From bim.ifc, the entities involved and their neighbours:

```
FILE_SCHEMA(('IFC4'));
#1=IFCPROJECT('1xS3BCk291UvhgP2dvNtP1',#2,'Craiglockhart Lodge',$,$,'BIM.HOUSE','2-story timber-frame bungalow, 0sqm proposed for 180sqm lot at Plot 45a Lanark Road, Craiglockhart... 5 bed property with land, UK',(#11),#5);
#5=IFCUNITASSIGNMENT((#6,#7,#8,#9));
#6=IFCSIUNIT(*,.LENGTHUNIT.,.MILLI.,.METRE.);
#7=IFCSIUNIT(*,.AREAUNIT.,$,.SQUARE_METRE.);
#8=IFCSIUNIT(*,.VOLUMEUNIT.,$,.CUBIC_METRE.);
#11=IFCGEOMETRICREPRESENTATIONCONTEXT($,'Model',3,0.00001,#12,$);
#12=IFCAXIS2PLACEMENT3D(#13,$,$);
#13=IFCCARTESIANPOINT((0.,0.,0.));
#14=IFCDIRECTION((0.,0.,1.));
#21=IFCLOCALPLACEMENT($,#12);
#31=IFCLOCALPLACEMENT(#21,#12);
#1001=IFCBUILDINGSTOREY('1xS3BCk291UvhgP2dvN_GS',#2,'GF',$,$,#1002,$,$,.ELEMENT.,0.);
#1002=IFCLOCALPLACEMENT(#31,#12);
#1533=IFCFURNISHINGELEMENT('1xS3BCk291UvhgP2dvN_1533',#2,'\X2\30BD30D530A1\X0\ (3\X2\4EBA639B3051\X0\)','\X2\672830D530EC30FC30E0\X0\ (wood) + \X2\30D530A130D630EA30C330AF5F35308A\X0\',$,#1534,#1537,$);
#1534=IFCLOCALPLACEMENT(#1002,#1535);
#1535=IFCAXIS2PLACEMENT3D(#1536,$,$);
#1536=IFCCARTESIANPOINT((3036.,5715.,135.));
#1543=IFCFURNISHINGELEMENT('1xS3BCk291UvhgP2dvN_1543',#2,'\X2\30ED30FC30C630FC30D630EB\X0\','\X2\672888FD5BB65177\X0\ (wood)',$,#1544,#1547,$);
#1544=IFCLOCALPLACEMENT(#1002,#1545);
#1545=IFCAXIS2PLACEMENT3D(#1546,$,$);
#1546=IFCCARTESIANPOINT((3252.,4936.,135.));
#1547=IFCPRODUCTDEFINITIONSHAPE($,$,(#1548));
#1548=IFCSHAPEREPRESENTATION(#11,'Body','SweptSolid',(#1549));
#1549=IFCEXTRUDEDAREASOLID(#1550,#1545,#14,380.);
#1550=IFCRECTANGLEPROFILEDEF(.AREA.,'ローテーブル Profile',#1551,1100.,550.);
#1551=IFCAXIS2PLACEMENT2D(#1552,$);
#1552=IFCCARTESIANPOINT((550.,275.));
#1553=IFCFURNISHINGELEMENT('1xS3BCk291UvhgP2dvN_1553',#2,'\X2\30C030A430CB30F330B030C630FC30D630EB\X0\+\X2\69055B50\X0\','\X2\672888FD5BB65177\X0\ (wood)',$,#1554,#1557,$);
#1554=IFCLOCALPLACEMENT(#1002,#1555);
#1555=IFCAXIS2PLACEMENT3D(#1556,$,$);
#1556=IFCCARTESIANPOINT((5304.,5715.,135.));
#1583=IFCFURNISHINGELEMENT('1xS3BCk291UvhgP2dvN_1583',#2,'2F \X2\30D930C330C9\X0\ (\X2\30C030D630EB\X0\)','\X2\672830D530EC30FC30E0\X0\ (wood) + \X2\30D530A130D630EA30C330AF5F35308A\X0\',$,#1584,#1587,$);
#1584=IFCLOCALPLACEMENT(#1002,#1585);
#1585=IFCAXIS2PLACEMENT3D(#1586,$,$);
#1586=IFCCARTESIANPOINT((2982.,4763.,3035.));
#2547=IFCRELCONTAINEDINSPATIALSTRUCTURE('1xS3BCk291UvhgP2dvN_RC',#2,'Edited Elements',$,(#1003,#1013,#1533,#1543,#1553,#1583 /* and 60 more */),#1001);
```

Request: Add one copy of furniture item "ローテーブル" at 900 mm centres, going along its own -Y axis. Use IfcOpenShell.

```python
import ifcopenshell
import ifcopenshell.api.geometry
import ifcopenshell.api.root
import ifcopenshell.util.element
import ifcopenshell.util.placement

model = ifcopenshell.open("bim.ifc")


def reuse_history(source, copy):
    """copy_class also copies each property set's owner history, people and application; keep the originals."""
    for rel in copy.IsDefinedBy:
        if rel.is_a("IfcRelDefinesByProperties") and (history := rel.RelatingPropertyDefinition.OwnerHistory):
            rel.RelatingPropertyDefinition.OwnerHistory = source.OwnerHistory
            ifcopenshell.util.element.remove_deep2(model, history)


source = model.by_id(1543)
base = ifcopenshell.util.placement.get_local_placement(source.ObjectPlacement)
step = -base[:3, 1] * 900.0

for i in range(1, 2):
    copy = ifcopenshell.api.root.copy_class(model, product=source)
    copy.Representation = ifcopenshell.util.element.copy_deep(
        model, source.Representation, exclude=["IfcGeometricRepresentationContext", "IfcRepresentationMap"]
    )
    reuse_history(source, copy)
    matrix = base.copy()
    matrix[:3, 3] += i * step
    print("added at", matrix[:3, 3].round(3) + 0.0)
    ifcopenshell.api.geometry.edit_object_placement(model, product=copy, matrix=matrix, is_si=False)

model.write("bim_rev.ifc")
```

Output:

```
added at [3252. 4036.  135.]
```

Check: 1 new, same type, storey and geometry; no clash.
